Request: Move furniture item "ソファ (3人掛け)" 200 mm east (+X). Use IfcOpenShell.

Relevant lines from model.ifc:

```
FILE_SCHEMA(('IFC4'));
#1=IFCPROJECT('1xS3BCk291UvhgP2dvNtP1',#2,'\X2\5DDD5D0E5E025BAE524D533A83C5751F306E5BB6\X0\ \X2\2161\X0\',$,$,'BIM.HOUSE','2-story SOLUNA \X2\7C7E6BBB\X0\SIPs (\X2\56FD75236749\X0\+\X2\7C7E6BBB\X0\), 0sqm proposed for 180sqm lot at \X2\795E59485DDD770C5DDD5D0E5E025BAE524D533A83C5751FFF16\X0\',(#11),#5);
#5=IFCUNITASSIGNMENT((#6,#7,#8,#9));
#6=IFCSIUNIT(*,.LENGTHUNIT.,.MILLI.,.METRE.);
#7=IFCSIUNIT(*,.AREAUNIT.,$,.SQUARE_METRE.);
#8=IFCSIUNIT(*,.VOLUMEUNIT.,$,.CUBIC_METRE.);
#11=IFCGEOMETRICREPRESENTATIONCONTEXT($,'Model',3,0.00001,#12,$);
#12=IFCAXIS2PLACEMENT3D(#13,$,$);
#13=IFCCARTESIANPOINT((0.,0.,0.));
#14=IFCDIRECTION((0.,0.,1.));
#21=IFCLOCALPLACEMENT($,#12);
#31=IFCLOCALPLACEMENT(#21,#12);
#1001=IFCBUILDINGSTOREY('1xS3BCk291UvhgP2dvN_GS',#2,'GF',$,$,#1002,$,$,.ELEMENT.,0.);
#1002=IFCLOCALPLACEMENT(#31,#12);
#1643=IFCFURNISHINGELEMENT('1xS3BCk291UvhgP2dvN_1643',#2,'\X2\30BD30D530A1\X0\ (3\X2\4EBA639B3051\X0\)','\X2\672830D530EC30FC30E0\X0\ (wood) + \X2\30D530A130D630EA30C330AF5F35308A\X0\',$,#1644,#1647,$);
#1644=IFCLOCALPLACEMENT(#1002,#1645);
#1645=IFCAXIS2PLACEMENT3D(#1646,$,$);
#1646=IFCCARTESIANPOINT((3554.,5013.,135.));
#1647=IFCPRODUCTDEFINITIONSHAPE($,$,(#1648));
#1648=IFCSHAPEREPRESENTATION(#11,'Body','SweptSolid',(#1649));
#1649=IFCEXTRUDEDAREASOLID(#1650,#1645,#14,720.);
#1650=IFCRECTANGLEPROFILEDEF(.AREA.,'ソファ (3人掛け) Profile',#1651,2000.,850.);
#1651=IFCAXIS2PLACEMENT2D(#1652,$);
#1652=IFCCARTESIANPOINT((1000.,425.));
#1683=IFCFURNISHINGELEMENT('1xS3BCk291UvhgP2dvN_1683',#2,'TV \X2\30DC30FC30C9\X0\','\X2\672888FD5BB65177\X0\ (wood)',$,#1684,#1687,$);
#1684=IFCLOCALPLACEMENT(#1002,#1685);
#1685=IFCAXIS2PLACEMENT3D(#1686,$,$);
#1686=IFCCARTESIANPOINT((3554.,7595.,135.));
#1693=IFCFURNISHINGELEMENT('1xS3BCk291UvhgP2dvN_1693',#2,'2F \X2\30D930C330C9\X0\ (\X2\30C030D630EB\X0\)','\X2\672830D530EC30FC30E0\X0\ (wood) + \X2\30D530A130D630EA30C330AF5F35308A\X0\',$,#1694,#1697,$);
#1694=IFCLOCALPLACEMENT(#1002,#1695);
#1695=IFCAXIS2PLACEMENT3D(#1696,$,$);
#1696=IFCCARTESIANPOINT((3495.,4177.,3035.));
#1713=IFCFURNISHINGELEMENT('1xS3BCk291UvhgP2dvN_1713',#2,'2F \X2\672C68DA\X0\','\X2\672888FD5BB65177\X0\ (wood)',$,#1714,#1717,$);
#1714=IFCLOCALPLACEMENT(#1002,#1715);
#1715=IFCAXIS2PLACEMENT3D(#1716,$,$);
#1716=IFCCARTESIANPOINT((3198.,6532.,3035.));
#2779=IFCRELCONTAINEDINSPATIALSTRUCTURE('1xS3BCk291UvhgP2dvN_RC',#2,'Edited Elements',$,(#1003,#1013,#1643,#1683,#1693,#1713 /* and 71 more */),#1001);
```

```python
import ifcopenshell
import ifcopenshell.api.geometry
import ifcopenshell.util.placement
import ifcopenshell.util.unit

model = ifcopenshell.open("model.ifc")
unit_scale = ifcopenshell.util.unit.calculate_unit_scale(model)

item = model.by_guid("1xS3BCk291UvhgP2dvN_1643")
matrix = ifcopenshell.util.placement.get_local_placement(item.ObjectPlacement)
matrix[0, 3] += 0.2 / unit_scale
ifcopenshell.api.geometry.edit_object_placement(model, product=item, matrix=matrix, is_si=False)

print(ifcopenshell.util.placement.get_local_placement(item.ObjectPlacement).round(3) + 0.0)

model.write("model_v2.ifc")
```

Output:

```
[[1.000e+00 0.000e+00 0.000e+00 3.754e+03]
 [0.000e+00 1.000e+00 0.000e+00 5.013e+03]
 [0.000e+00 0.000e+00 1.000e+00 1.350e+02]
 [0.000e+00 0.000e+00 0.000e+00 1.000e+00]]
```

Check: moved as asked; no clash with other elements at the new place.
